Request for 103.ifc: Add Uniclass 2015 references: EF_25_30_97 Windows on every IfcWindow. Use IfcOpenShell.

First a look at what the model holds.

```python
import ifcopenshell

model = ifcopenshell.open("103.ifc")
print(model.schema)
print("classifications:", [c.Name for c in model.by_type("IfcClassification")])
for ifc_class in ("IfcDoor", "IfcRoof", "IfcStair", "IfcWall", "IfcWindow"):
    print(ifc_class, len(model.by_type(ifc_class)))
```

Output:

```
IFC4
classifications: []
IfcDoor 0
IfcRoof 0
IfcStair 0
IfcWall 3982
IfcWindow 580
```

```python
import ifcopenshell
import ifcopenshell.api.classification

model = ifcopenshell.open("103.ifc")

system = ifcopenshell.api.classification.add_classification(model, classification="Uniclass 2015")

codes = {
    "IfcWindow": ("EF_25_30_97", "Windows"),
}
for ifc_class, (code, name) in codes.items():
    products = model.by_type(ifc_class)
    ifcopenshell.api.classification.add_reference(
        model, products=products, classification=system, identification=code, name=name
    )
    print(code, len(products))

model.write("103_updated.ifc")
```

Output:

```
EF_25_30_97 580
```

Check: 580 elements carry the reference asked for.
